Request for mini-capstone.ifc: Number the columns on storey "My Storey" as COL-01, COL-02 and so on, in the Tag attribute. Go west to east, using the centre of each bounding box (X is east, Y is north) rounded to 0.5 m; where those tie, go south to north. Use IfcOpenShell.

First a look at what the model holds.

```python
import ifcopenshell
import ifcopenshell.util.element
import ifcopenshell.util.placement

model = ifcopenshell.open("mini-capstone.ifc")
print(model.schema)
storey = next(s for s in model.by_type("IfcBuildingStorey") if s.Name == "My Storey")
columns = [e for e in ifcopenshell.util.element.get_decomposition(storey) if e.is_a("IfcColumn")]
for e in sorted(columns, key=lambda e: e.id()):
    origin = ifcopenshell.util.placement.get_local_placement(e.ObjectPlacement)[:3, 3]
    print(e.id(), e.Tag, e.Name, origin.round(2) + 0.0, sep=" | ")
```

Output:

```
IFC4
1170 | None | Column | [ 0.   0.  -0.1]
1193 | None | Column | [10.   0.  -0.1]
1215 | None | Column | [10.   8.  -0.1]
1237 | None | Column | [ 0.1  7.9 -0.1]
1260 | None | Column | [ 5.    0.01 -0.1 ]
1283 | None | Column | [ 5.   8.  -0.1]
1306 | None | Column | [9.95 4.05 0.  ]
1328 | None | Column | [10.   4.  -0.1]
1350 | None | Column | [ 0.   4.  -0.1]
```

```python
import ifcopenshell
import ifcopenshell.geom
import ifcopenshell.util.element
import ifcopenshell.util.shape

model = ifcopenshell.open("mini-capstone.ifc")
settings = ifcopenshell.geom.settings()
settings.set("use-world-coords", True)


def centre(element):
    shape = ifcopenshell.geom.create_shape(settings, element)
    return ifcopenshell.util.shape.get_bbox_centroid(shape.geometry)


storey = next(s for s in model.by_type("IfcBuildingStorey") if s.Name == "My Storey")
columns = [e for e in ifcopenshell.util.element.get_decomposition(storey) if e.is_a("IfcColumn")]

# Insertion points can sit at a corner or the storey origin, so sort by the geometry (in metres).
centres = {e: centre(e) for e in columns}
columns.sort(key=lambda e: (round(centres[e][0] / 0.5), centres[e][1]))

for i, e in enumerate(columns, start=1):
    number = f"COL-{i:02d}"
    e.Tag = number
    print(e.id(), number)

model.write("mini-capstone_v2.ifc")
```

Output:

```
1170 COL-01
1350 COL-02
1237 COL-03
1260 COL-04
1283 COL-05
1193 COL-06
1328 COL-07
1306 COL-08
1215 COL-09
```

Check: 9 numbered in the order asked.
